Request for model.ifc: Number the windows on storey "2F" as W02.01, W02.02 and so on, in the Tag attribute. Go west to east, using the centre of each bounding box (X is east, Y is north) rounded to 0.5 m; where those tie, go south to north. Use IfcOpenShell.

First a look at what the model holds.

```python
import ifcopenshell
import ifcopenshell.util.element
import ifcopenshell.util.placement

model = ifcopenshell.open("model.ifc")
print(model.schema)
storey = next(s for s in model.by_type("IfcBuildingStorey") if s.Name == "2F")
windows = [e for e in ifcopenshell.util.element.get_decomposition(storey) if e.is_a("IfcWindow")]
for e in sorted(windows, key=lambda e: e.id()):
    origin = ifcopenshell.util.placement.get_local_placement(e.ObjectPlacement)[:3, 3]
    print(e.id(), e.Tag, e.Name, origin.round(2) + 0.0, sep=" | ")
```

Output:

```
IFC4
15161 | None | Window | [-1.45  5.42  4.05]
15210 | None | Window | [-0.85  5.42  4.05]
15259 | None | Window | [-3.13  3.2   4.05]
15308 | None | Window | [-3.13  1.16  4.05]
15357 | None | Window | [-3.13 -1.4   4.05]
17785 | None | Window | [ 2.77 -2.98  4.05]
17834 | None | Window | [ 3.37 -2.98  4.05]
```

```python
import ifcopenshell
import ifcopenshell.geom
import ifcopenshell.util.element
import ifcopenshell.util.shape

model = ifcopenshell.open("model.ifc")
settings = ifcopenshell.geom.settings()
settings.set("use-world-coords", True)


def centre(element):
    shape = ifcopenshell.geom.create_shape(settings, element)
    return ifcopenshell.util.shape.get_bbox_centroid(shape.geometry)


storey = next(s for s in model.by_type("IfcBuildingStorey") if s.Name == "2F")
windows = [e for e in ifcopenshell.util.element.get_decomposition(storey) if e.is_a("IfcWindow")]

# Insertion points can sit at a corner or the storey origin, so sort by the geometry (in metres).
centres = {e: centre(e) for e in windows}
windows.sort(key=lambda e: (round(centres[e][0] / 0.5), centres[e][1]))

for i, e in enumerate(windows, start=1):
    number = f"W02.{i:02d}"
    e.Tag = number
    print(e.id(), number)

model.write("model_v2.ifc")
```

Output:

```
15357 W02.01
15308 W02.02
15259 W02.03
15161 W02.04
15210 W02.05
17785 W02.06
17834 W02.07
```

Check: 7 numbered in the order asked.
